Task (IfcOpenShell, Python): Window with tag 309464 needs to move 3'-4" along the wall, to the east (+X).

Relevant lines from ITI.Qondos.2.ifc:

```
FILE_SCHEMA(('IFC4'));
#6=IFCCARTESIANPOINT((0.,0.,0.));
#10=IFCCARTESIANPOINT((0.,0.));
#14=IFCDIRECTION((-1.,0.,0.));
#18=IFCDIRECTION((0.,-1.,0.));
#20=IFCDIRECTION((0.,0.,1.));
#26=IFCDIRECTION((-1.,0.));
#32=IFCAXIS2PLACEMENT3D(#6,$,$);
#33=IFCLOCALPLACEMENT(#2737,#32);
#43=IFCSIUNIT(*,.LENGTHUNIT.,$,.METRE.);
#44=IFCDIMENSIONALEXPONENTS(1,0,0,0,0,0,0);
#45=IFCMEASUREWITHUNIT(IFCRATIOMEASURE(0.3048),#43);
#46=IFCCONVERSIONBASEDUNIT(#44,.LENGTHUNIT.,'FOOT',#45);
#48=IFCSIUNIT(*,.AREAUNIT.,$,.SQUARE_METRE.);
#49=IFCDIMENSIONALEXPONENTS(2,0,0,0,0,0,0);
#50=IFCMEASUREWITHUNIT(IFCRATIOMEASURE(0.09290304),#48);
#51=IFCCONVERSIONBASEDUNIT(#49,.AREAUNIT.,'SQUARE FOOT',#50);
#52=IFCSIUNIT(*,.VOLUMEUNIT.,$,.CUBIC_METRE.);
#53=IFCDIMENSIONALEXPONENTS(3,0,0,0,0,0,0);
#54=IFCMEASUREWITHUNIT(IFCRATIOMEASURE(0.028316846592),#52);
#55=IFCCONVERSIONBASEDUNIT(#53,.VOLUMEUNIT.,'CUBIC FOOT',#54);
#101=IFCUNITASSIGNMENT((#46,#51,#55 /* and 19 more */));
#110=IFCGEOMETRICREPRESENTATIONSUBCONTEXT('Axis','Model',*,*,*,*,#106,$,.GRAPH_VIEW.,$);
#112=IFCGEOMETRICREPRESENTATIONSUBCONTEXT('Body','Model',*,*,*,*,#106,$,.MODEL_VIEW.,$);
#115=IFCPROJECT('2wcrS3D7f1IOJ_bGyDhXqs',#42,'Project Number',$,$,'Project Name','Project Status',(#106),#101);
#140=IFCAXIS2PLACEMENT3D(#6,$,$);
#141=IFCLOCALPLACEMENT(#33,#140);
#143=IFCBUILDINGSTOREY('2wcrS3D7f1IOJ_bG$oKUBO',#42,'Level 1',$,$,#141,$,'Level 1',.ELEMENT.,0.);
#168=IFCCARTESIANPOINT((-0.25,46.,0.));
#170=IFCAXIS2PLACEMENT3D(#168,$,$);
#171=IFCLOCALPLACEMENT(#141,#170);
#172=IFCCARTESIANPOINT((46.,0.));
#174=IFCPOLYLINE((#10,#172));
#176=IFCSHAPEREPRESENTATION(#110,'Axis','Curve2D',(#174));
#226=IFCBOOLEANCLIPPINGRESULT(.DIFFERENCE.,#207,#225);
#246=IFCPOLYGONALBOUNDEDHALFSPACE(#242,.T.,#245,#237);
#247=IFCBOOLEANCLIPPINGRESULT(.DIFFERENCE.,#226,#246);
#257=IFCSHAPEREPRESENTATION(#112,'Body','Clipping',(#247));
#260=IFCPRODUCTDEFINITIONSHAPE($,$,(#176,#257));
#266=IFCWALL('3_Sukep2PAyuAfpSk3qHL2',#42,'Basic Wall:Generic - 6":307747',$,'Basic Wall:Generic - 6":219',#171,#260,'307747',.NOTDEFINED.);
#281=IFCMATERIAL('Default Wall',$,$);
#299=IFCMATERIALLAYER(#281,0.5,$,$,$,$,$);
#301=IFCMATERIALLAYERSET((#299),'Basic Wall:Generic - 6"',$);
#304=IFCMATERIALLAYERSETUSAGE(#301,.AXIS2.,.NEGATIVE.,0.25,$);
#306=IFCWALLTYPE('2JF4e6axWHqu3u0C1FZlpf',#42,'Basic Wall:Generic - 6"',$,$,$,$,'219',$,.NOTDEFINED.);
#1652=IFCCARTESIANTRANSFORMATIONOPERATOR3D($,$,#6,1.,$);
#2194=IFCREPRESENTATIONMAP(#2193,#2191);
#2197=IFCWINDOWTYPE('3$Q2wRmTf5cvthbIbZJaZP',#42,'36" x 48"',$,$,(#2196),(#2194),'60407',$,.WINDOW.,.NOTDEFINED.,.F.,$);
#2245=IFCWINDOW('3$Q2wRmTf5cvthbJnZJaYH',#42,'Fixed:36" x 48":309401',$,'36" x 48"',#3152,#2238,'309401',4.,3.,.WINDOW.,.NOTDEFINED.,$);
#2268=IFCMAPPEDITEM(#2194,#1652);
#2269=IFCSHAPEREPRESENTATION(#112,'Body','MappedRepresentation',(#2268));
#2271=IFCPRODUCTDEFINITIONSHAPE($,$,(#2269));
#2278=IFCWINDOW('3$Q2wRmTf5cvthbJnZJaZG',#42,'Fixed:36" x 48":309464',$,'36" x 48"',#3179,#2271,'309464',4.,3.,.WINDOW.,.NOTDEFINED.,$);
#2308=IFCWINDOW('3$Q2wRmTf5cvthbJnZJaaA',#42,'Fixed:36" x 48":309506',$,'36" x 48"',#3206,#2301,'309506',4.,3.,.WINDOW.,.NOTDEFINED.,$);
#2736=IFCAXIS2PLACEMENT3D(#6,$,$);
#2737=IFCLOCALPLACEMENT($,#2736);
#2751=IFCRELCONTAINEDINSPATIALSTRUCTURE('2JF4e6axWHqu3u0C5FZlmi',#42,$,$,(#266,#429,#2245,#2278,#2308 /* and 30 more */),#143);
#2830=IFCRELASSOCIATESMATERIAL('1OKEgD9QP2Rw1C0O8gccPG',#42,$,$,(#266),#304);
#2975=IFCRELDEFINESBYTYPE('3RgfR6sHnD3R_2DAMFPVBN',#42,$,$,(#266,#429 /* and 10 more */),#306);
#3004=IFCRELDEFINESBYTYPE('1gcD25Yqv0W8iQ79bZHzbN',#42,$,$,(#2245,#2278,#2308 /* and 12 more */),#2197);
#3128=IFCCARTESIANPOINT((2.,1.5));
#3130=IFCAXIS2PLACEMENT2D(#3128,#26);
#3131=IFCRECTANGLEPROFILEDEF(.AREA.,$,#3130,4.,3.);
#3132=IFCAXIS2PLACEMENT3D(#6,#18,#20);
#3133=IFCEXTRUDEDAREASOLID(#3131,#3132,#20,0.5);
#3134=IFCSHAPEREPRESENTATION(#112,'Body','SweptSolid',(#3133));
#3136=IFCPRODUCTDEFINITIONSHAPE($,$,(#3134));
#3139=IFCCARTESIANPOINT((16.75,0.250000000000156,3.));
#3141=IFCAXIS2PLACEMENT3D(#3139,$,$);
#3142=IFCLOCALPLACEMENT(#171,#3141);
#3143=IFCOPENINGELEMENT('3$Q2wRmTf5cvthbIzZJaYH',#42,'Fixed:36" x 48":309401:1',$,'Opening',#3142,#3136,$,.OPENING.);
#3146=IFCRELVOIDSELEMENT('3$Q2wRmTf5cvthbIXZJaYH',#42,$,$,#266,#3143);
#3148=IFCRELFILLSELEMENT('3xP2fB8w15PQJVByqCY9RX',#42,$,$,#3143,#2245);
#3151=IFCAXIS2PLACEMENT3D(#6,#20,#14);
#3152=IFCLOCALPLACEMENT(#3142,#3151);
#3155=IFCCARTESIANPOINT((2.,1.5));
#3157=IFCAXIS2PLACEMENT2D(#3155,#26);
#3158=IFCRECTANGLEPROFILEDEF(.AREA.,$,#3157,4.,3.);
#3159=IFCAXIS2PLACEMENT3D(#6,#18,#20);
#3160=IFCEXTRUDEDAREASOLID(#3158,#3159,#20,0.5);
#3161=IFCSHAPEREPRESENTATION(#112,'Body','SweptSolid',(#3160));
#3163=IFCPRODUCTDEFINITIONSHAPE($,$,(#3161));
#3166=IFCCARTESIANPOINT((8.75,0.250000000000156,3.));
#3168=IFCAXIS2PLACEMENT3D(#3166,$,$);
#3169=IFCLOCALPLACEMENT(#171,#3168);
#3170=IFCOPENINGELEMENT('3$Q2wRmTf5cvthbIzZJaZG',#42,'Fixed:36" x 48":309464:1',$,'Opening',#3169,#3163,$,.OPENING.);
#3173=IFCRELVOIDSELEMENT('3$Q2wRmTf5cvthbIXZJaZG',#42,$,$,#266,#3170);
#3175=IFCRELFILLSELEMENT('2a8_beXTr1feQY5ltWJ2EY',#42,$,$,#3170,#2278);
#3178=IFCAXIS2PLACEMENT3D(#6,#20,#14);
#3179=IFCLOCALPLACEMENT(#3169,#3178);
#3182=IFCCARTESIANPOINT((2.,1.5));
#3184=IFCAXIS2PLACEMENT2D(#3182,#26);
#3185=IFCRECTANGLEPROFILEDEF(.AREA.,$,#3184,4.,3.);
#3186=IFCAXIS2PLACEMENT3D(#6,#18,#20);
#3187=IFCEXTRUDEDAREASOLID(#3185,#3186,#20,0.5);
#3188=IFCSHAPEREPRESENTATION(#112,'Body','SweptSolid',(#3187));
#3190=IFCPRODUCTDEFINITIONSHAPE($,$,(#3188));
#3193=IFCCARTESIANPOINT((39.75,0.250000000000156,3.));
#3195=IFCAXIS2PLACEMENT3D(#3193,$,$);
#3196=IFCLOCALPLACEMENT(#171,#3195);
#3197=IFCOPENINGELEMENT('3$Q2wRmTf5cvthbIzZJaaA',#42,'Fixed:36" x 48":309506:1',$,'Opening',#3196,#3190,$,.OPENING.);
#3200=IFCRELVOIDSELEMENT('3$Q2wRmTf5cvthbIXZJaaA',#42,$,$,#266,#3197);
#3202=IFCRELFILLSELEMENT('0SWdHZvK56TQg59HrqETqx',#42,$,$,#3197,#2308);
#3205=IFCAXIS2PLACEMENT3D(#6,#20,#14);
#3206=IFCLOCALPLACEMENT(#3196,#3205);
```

```python
import ifcopenshell
import ifcopenshell.api.geometry
import ifcopenshell.util.placement
import ifcopenshell.util.unit

model = ifcopenshell.open("ITI.Qondos.2.ifc")
unit_scale = ifcopenshell.util.unit.calculate_unit_scale(model)

window = model.by_id(2278)
opening = window.FillsVoids[0].RelatingOpeningElement
wall = opening.VoidsElements[0].RelatingBuildingElement

wall_matrix = ifcopenshell.util.placement.get_local_placement(wall.ObjectPlacement)
shift = wall_matrix[:3, 0] * 40 * 0.0254 / unit_scale
before = ifcopenshell.util.placement.get_local_placement(window.ObjectPlacement)[:3, 3].copy()

# The window is placed relative to its opening, so it follows when the opening moves.
matrix = ifcopenshell.util.placement.get_local_placement(opening.ObjectPlacement)
matrix[:3, 3] += shift
ifcopenshell.api.geometry.edit_object_placement(
    model, product=opening, matrix=matrix, is_si=False, should_transform_children=True
)

after = ifcopenshell.util.placement.get_local_placement(window.ObjectPlacement)[:3, 3]
print("window moved by", (after - before).round(3) + 0.0)

model.write("ITI.Qondos.2_rev.ifc")
```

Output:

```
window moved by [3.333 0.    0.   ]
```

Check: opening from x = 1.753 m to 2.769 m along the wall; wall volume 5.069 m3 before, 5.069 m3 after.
